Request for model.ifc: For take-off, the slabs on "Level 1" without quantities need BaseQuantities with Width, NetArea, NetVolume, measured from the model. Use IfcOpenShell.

First a look at what the model holds.

```python
import ifcopenshell
import ifcopenshell.util.element
import ifcopenshell.util.unit

model = ifcopenshell.open("model.ifc")
print(model.schema)
for unit_type in ("LENGTHUNIT", "AREAUNIT", "VOLUMEUNIT"):
    print(unit_type, ifcopenshell.util.unit.calculate_unit_scale(model, unit_type))
storey = next(s for s in model.by_type("IfcBuildingStorey") if s.Name == "Level 1")
slabs = [e for e in ifcopenshell.util.element.get_decomposition(storey) if e.is_a("IfcSlab")]
for e in sorted(slabs, key=lambda e: e.id()):
    print(e.id(), e.is_a(), e.Name, list(ifcopenshell.util.element.get_psets(e, qtos_only=True)), sep=" | ")
```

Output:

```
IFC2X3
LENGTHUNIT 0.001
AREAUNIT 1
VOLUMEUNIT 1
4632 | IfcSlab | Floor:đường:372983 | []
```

```python
import ifcopenshell
import ifcopenshell.api.pset
import ifcopenshell.geom
import ifcopenshell.util.element
import ifcopenshell.util.shape
import ifcopenshell.util.unit

model = ifcopenshell.open("model.ifc")
unit_scale = ifcopenshell.util.unit.calculate_unit_scale(model)
area_scale = ifcopenshell.util.unit.calculate_unit_scale(model, "AREAUNIT")
volume_scale = ifcopenshell.util.unit.calculate_unit_scale(model, "VOLUMEUNIT")
settings = ifcopenshell.geom.settings()

storey = next(s for s in model.by_type("IfcBuildingStorey") if s.Name == "Level 1")
slabs = [e for e in ifcopenshell.util.element.get_decomposition(storey) if e.is_a("IfcSlab")]

for e in sorted(slabs, key=lambda e: e.id()):
    if ifcopenshell.util.element.get_psets(e, qtos_only=True, should_inherit=False):
        continue
    # Geometry comes back in metres, in the element's own axes.
    shape = ifcopenshell.geom.create_shape(settings, e)
    values = {
        "Width": ifcopenshell.util.shape.get_z(shape.geometry) / unit_scale,
        "NetArea": ifcopenshell.util.shape.get_footprint_area(shape.geometry) / area_scale,
        "NetVolume": ifcopenshell.util.shape.get_volume(shape.geometry) / volume_scale,
    }
    qto = ifcopenshell.api.pset.add_qto(model, product=e, name="BaseQuantities")
    ifcopenshell.api.pset.edit_qto(model, qto=qto, properties=values)
    print(e.id(), {k: round(v, 3) for k, v in values.items()})

model.write("model_v2.ifc")
```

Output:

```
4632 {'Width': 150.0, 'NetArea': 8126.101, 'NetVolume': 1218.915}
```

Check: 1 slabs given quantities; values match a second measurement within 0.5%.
